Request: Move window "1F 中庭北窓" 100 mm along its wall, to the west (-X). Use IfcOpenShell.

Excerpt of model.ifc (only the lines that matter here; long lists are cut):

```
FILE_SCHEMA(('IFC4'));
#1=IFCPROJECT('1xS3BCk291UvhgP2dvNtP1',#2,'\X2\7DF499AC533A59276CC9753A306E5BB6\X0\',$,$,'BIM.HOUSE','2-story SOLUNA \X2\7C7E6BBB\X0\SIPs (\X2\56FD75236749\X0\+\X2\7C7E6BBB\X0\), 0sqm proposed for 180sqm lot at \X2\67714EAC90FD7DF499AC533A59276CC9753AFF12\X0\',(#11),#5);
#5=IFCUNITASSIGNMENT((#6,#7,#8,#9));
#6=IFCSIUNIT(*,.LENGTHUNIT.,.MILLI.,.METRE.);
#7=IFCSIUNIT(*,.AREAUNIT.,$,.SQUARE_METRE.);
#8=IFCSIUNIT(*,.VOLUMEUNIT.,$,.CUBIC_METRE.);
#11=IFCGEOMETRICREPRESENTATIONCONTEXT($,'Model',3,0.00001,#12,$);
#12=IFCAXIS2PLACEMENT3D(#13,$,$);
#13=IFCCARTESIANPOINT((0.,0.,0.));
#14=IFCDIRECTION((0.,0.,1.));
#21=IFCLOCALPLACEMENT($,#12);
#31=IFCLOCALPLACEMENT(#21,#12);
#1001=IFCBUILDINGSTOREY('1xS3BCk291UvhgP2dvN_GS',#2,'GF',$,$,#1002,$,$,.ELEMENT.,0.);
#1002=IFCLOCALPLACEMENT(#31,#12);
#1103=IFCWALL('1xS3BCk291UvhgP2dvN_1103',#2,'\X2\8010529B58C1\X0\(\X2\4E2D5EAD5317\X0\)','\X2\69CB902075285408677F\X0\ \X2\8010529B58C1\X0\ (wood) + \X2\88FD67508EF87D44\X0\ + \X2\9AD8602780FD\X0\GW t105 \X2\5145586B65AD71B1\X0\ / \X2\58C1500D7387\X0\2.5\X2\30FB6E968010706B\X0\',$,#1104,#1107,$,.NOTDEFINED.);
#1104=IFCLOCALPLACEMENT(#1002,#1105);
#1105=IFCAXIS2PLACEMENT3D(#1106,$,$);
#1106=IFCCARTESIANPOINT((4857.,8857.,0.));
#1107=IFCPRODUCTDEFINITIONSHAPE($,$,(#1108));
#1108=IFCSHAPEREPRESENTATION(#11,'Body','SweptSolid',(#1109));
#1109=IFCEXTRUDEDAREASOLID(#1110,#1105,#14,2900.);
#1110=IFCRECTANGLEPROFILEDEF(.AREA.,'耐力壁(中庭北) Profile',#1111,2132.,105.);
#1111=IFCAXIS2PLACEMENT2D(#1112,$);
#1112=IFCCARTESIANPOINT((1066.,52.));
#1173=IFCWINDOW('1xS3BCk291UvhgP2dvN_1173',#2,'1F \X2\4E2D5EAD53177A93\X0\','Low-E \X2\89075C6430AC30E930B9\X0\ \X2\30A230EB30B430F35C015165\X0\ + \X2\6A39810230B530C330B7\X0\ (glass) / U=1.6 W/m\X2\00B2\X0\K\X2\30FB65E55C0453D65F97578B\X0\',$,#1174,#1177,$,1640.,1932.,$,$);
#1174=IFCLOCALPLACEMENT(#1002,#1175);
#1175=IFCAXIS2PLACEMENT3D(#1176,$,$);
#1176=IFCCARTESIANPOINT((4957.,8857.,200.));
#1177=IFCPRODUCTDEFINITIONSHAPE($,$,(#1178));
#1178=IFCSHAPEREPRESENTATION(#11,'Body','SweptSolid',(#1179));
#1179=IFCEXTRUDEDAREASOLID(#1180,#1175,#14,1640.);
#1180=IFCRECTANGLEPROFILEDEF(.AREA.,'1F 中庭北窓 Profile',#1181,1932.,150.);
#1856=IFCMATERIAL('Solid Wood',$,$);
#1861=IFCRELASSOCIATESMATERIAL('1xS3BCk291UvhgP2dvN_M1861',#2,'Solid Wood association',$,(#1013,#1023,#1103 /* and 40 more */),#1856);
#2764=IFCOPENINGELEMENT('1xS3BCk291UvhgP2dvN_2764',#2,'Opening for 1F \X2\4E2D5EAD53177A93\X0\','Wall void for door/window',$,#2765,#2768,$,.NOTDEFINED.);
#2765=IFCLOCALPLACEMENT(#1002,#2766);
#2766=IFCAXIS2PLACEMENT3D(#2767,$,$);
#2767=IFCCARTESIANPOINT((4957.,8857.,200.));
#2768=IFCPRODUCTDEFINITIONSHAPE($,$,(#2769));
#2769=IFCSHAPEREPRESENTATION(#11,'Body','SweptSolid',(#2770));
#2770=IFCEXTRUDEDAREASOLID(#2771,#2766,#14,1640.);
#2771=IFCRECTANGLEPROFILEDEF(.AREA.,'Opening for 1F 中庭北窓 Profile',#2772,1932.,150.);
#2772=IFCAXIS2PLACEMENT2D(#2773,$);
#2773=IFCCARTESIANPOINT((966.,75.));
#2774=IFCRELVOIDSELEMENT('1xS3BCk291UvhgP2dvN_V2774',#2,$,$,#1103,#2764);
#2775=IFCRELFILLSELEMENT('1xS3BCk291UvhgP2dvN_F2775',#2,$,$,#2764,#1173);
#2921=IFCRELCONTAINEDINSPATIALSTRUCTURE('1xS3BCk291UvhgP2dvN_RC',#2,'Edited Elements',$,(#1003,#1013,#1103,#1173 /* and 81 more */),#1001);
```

```python
import ifcopenshell
import ifcopenshell.api.geometry
import ifcopenshell.util.placement
import ifcopenshell.util.unit

model = ifcopenshell.open("model.ifc")
unit_scale = ifcopenshell.util.unit.calculate_unit_scale(model)

window = model.by_guid("1xS3BCk291UvhgP2dvN_1173")
opening = window.FillsVoids[0].RelatingOpeningElement
wall = opening.VoidsElements[0].RelatingBuildingElement

wall_matrix = ifcopenshell.util.placement.get_local_placement(wall.ObjectPlacement)
shift = wall_matrix[:3, 0] * -0.1 / unit_scale
before = ifcopenshell.util.placement.get_local_placement(window.ObjectPlacement)[:3, 3].copy()

# The window is not placed relative to its opening, so move both.
for product in (opening, window):
    matrix = ifcopenshell.util.placement.get_local_placement(product.ObjectPlacement)
    matrix[:3, 3] += shift
    ifcopenshell.api.geometry.edit_object_placement(model, product=product, matrix=matrix, is_si=False)

after = ifcopenshell.util.placement.get_local_placement(window.ObjectPlacement)[:3, 3]
print("window moved by", (after - before).round(3) + 0.0)

model.write("model_rev.ifc")
```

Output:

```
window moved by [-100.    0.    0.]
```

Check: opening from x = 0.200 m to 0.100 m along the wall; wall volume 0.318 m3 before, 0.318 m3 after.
